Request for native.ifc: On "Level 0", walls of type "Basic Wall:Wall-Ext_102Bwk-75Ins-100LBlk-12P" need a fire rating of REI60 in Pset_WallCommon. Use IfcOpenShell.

First a look at what the model holds.

```python
import ifcopenshell
import ifcopenshell.util.element

model = ifcopenshell.open("native.ifc")
print(model.schema)
storey = next(s for s in model.by_type("IfcBuildingStorey") if s.Name == "Level 0")
walls = [e for e in ifcopenshell.util.element.get_decomposition(storey) if e.is_a("IfcWall")]
seen = {}
for e in walls:
    element_type = ifcopenshell.util.element.get_type(e)
    key = (element_type.Name if element_type != e and element_type else None, ifcopenshell.util.element.get_pset(e, "Pset_WallCommon", "FireRating"))
    seen[key] = seen.get(key, 0) + 1
for (name, value), count in sorted(seen.items(), key=str):
    print(count, "x", name, "|", value)
```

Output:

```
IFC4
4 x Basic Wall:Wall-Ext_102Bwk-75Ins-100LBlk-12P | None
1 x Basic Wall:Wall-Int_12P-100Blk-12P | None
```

```python
import ifcopenshell
import ifcopenshell.api.pset
import ifcopenshell.util.element

model = ifcopenshell.open("native.ifc")

storey = next(s for s in model.by_type("IfcBuildingStorey") if s.Name == "Level 0")
walls = [e for e in ifcopenshell.util.element.get_decomposition(storey) if e.is_a("IfcWall")]

count = 0
for e in walls:
    element_type = ifcopenshell.util.element.get_type(e)
    if element_type in (None, e) or element_type.Name != "Basic Wall:Wall-Ext_102Bwk-75Ins-100LBlk-12P":
        continue
    # add_pset returns the element's existing set when there is one.
    pset = ifcopenshell.api.pset.add_pset(model, product=e, name="Pset_WallCommon")
    ifcopenshell.api.pset.edit_pset(model, pset=pset, properties={"FireRating": "REI60"})
    count += 1

print(count, "walls updated")

model.write("native_updated.ifc")
```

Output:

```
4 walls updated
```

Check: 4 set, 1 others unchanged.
